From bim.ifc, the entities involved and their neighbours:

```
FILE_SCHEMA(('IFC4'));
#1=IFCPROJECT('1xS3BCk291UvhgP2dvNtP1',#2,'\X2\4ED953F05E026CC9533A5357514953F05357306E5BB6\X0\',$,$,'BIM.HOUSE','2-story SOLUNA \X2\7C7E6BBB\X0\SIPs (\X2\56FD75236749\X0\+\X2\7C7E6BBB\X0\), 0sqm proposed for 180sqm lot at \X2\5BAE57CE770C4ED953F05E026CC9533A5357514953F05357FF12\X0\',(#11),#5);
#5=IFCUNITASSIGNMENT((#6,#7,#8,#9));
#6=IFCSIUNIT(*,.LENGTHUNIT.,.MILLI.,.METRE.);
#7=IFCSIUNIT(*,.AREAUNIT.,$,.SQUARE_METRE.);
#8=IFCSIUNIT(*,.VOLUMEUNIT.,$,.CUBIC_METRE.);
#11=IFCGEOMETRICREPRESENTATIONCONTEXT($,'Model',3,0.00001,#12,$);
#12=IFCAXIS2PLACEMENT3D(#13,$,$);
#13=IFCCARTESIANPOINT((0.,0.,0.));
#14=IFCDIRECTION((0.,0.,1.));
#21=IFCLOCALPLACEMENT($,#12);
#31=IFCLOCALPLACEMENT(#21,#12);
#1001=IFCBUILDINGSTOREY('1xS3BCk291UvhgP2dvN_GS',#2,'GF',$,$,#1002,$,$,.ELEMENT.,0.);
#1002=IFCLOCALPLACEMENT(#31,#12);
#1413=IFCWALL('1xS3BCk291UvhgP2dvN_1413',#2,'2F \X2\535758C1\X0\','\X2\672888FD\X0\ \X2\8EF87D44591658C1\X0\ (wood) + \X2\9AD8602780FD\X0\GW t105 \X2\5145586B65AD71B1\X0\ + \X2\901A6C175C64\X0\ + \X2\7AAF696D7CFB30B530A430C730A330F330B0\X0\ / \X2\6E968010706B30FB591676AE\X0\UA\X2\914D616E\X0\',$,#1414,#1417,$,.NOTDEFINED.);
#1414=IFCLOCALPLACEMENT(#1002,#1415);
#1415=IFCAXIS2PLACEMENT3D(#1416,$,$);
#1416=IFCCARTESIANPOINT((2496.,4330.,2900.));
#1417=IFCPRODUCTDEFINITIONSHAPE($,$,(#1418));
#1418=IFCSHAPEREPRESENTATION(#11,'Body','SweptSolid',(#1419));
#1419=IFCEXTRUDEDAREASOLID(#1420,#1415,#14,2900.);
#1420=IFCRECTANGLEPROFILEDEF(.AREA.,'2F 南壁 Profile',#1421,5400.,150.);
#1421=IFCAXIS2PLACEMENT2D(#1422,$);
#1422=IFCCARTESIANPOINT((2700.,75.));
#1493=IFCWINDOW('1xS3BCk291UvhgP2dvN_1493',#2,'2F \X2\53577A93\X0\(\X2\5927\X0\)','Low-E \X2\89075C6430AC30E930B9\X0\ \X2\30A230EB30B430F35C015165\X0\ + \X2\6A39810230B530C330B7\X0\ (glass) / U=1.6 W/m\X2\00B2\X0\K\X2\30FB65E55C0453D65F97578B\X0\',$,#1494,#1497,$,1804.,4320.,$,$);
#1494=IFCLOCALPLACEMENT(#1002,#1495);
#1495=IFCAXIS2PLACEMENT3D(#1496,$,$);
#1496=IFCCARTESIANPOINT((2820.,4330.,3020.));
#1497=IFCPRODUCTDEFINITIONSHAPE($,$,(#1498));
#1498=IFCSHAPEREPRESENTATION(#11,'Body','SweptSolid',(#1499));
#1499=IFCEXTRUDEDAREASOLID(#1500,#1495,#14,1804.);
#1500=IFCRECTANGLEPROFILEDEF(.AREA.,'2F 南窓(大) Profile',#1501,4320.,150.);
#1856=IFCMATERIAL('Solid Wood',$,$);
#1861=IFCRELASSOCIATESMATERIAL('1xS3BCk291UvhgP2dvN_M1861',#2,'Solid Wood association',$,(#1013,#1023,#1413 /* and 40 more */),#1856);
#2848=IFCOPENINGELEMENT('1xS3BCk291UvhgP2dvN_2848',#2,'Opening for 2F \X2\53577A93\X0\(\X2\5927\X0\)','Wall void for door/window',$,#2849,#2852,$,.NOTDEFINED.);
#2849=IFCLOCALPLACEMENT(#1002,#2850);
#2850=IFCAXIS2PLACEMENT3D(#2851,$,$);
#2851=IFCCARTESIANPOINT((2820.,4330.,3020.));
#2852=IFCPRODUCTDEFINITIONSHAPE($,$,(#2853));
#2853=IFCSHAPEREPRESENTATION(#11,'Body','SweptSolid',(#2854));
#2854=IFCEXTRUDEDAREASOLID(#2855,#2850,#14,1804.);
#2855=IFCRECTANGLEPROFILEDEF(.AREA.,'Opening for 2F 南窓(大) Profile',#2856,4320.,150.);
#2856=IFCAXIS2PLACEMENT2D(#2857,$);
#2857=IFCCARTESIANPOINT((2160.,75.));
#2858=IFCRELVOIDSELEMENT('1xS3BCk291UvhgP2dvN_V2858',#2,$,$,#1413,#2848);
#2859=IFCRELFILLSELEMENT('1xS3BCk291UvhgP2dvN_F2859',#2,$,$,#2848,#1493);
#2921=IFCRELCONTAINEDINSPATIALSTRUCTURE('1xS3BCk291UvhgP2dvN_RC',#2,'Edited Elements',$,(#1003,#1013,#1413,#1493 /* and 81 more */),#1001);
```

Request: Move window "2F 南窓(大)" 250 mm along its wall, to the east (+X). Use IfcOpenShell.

```python
import ifcopenshell
import ifcopenshell.api.geometry
import ifcopenshell.util.placement
import ifcopenshell.util.unit

model = ifcopenshell.open("bim.ifc")
unit_scale = ifcopenshell.util.unit.calculate_unit_scale(model)

window = model.by_guid("1xS3BCk291UvhgP2dvN_1493")
opening = window.FillsVoids[0].RelatingOpeningElement
wall = opening.VoidsElements[0].RelatingBuildingElement

wall_matrix = ifcopenshell.util.placement.get_local_placement(wall.ObjectPlacement)
shift = wall_matrix[:3, 0] * 0.25 / unit_scale
before = ifcopenshell.util.placement.get_local_placement(window.ObjectPlacement)[:3, 3].copy()

# The window is not placed relative to its opening, so move both.
for product in (opening, window):
    matrix = ifcopenshell.util.placement.get_local_placement(product.ObjectPlacement)
    matrix[:3, 3] += shift
    ifcopenshell.api.geometry.edit_object_placement(model, product=product, matrix=matrix, is_si=False)

after = ifcopenshell.util.placement.get_local_placement(window.ObjectPlacement)[:3, 3]
print("window moved by", (after - before).round(3) + 0.0)

model.write("bim_rev.ifc")
```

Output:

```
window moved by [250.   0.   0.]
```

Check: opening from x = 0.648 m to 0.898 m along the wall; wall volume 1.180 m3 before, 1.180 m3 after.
